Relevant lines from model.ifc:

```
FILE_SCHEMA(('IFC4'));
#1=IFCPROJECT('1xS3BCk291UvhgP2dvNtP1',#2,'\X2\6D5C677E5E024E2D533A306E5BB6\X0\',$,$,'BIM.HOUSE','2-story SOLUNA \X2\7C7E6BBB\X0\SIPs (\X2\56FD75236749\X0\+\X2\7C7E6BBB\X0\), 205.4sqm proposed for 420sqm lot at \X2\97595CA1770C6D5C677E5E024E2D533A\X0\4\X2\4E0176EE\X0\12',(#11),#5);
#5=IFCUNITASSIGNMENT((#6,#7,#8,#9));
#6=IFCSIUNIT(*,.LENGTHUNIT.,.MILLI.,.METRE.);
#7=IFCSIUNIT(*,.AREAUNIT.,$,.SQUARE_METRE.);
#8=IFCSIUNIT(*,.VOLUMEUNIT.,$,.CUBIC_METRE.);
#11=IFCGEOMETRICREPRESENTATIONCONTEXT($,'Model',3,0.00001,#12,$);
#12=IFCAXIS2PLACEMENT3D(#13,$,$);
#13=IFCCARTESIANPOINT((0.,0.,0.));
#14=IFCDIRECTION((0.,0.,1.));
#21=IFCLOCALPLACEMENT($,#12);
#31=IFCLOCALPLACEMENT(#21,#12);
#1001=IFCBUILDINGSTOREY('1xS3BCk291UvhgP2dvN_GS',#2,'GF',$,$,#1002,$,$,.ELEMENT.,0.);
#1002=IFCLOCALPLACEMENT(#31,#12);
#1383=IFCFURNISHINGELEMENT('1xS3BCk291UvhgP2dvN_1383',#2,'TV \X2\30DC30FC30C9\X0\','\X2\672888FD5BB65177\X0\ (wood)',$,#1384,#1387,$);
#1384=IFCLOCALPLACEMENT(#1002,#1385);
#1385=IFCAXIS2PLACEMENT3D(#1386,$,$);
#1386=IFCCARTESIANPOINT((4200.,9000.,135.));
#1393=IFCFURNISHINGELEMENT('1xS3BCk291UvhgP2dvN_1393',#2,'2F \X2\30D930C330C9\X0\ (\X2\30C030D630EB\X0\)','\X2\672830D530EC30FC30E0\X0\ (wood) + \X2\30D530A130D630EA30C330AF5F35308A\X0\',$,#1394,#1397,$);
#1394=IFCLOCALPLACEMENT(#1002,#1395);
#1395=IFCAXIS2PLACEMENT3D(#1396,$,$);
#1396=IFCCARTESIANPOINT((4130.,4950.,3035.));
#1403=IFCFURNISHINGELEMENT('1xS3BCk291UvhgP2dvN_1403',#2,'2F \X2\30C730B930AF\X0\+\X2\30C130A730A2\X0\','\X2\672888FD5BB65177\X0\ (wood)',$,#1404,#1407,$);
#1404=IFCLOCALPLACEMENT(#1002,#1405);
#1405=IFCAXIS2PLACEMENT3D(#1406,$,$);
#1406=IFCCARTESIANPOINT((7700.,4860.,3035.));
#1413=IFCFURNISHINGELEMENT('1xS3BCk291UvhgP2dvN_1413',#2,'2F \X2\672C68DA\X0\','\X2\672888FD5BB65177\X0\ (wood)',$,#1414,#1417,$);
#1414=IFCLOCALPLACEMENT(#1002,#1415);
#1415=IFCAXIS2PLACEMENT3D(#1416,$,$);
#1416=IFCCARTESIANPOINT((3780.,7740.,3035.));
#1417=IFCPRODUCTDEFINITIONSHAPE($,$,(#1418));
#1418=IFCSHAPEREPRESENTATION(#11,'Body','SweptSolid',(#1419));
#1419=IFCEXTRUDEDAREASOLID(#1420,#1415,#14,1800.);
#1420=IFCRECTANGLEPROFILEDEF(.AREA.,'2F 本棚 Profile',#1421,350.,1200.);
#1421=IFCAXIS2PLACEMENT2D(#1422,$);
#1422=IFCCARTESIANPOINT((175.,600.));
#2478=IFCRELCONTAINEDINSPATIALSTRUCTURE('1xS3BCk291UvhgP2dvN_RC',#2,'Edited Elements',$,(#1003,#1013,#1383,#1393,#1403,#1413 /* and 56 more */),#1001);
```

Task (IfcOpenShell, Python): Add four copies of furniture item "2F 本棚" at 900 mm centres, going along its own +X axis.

```python
import ifcopenshell
import ifcopenshell.api.geometry
import ifcopenshell.api.root
import ifcopenshell.util.element
import ifcopenshell.util.placement

model = ifcopenshell.open("model.ifc")


def reuse_history(source, copy):
    """copy_class also copies each property set's owner history, people and application; keep the originals."""
    for rel in copy.IsDefinedBy:
        if rel.is_a("IfcRelDefinesByProperties") and (history := rel.RelatingPropertyDefinition.OwnerHistory):
            rel.RelatingPropertyDefinition.OwnerHistory = source.OwnerHistory
            ifcopenshell.util.element.remove_deep2(model, history)


source = model.by_id(1413)
base = ifcopenshell.util.placement.get_local_placement(source.ObjectPlacement)
step = base[:3, 0] * 900.0

for i in range(1, 5):
    copy = ifcopenshell.api.root.copy_class(model, product=source)
    copy.Representation = ifcopenshell.util.element.copy_deep(
        model, source.Representation, exclude=["IfcGeometricRepresentationContext", "IfcRepresentationMap"]
    )
    reuse_history(source, copy)
    matrix = base.copy()
    matrix[:3, 3] += i * step
    print("added at", matrix[:3, 3].round(3) + 0.0)
    ifcopenshell.api.geometry.edit_object_placement(model, product=copy, matrix=matrix, is_si=False)

model.write("model_updated.ifc")
```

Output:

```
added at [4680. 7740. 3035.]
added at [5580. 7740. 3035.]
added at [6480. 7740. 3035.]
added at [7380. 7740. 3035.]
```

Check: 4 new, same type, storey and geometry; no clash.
